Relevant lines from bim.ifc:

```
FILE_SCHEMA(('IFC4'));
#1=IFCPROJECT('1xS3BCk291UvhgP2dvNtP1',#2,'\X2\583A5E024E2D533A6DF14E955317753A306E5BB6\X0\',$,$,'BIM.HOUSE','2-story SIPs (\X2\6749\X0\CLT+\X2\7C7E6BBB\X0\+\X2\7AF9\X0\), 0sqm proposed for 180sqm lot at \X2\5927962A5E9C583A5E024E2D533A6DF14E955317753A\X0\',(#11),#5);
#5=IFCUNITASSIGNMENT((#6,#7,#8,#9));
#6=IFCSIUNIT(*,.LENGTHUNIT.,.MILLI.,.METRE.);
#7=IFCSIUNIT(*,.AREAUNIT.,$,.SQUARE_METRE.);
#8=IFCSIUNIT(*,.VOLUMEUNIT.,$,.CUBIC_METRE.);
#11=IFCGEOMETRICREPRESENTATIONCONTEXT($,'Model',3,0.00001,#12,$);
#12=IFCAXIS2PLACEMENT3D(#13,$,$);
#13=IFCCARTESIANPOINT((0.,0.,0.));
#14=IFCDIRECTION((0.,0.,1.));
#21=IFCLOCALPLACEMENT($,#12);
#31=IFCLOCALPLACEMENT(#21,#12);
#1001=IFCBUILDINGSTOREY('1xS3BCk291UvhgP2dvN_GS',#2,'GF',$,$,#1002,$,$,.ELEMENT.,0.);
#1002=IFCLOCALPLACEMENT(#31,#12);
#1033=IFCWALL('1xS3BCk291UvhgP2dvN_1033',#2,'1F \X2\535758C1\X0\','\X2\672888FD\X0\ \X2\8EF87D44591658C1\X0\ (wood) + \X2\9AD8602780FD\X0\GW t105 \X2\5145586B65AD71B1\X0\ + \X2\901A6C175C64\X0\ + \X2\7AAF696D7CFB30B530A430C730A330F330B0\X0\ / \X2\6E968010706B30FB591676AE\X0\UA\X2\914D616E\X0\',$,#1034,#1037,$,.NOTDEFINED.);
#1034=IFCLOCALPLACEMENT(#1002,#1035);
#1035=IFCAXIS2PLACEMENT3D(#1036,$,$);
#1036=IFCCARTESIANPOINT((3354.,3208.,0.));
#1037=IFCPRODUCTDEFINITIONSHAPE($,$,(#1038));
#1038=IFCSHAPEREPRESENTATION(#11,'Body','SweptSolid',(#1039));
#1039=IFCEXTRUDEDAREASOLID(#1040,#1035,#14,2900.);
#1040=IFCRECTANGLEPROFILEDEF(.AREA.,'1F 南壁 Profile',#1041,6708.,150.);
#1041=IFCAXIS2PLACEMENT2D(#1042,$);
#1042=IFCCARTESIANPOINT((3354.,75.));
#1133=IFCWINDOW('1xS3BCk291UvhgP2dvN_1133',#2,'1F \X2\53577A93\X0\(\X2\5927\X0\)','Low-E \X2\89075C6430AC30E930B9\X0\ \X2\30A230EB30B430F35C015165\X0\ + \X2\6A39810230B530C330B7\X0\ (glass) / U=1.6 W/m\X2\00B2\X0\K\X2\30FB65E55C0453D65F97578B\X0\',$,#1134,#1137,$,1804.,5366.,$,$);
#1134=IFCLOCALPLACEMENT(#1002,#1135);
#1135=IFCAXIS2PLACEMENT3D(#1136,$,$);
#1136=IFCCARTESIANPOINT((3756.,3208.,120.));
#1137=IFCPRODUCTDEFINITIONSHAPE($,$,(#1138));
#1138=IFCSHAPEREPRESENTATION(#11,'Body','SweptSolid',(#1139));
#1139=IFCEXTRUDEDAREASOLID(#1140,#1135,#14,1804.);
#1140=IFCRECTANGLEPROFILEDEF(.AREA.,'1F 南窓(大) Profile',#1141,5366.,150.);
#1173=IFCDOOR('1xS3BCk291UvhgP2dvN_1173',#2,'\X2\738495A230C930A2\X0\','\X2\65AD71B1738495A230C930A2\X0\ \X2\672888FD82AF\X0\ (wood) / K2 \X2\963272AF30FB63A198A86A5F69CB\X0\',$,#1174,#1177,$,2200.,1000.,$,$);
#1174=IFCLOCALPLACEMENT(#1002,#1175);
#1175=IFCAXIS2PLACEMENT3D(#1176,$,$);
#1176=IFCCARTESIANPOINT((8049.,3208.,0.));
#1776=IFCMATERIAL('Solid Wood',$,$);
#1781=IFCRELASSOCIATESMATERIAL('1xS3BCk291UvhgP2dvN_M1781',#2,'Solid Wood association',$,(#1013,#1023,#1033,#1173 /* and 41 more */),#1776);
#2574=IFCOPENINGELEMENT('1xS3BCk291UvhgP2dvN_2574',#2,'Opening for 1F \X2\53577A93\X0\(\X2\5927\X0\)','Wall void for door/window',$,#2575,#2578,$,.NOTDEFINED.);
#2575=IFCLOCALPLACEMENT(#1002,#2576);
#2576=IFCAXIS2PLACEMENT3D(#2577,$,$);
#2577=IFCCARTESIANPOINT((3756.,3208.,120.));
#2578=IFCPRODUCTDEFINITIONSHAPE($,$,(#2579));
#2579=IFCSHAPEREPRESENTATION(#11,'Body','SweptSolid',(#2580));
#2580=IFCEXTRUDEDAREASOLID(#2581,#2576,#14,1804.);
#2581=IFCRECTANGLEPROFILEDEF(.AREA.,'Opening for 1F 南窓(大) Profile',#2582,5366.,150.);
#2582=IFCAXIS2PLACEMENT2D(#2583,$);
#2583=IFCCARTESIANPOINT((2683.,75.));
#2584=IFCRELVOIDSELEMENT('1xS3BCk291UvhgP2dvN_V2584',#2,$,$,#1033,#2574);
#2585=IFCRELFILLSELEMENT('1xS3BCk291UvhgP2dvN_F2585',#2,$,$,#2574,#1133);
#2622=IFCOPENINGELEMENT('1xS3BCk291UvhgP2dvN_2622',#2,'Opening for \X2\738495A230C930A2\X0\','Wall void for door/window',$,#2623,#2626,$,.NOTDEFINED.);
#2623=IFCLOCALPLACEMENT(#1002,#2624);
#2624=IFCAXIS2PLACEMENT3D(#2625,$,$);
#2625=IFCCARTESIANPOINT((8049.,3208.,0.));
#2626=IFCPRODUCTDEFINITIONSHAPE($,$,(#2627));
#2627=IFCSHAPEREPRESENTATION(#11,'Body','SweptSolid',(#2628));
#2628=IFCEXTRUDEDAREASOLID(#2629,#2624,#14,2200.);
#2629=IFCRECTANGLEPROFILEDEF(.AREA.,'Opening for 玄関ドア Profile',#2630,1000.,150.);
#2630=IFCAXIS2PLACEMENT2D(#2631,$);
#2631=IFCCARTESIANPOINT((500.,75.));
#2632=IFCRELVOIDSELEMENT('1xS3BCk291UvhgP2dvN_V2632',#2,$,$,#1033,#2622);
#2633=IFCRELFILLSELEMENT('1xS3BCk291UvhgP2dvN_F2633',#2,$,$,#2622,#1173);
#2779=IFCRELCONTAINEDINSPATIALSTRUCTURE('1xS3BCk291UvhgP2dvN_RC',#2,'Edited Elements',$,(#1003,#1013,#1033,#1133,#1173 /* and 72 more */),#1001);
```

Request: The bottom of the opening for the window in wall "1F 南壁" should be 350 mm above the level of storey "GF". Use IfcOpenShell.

```python
import numpy as np
import ifcopenshell
import ifcopenshell.api.geometry
import ifcopenshell.geom
import ifcopenshell.util.element
import ifcopenshell.util.placement
import ifcopenshell.util.shape
import ifcopenshell.util.unit

model = ifcopenshell.open("bim.ifc")
unit_scale = ifcopenshell.util.unit.calculate_unit_scale(model)

window = model.by_guid("1xS3BCk291UvhgP2dvN_1133")
opening = window.FillsVoids[0].RelatingOpeningElement
storey = ifcopenshell.util.element.get_container(window, ifc_class="IfcBuildingStorey")
level = ifcopenshell.util.placement.get_local_placement(storey.ObjectPlacement)[2, 3]

# The opening's origin need not be at the sill, so measure its lowest point.
shape = ifcopenshell.geom.create_shape(ifcopenshell.geom.settings(), opening)
bottom = ifcopenshell.util.shape.get_shape_bottom_elevation(shape, shape.geometry) / unit_scale
dz = level + 0.35 / unit_scale - bottom

shift = np.array([0.0, 0.0, dz])
# The window is not placed relative to its opening, so move both.
for product in (opening, window):
    matrix = ifcopenshell.util.placement.get_local_placement(product.ObjectPlacement)
    matrix[:3, 3] += shift
    ifcopenshell.api.geometry.edit_object_placement(model, product=product, matrix=matrix, is_si=False)

print(f"moved by {dz * unit_scale:+.3f} m")

model.write("bim_v2.ifc")
```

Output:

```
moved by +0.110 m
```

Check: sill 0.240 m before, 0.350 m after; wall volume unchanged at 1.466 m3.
